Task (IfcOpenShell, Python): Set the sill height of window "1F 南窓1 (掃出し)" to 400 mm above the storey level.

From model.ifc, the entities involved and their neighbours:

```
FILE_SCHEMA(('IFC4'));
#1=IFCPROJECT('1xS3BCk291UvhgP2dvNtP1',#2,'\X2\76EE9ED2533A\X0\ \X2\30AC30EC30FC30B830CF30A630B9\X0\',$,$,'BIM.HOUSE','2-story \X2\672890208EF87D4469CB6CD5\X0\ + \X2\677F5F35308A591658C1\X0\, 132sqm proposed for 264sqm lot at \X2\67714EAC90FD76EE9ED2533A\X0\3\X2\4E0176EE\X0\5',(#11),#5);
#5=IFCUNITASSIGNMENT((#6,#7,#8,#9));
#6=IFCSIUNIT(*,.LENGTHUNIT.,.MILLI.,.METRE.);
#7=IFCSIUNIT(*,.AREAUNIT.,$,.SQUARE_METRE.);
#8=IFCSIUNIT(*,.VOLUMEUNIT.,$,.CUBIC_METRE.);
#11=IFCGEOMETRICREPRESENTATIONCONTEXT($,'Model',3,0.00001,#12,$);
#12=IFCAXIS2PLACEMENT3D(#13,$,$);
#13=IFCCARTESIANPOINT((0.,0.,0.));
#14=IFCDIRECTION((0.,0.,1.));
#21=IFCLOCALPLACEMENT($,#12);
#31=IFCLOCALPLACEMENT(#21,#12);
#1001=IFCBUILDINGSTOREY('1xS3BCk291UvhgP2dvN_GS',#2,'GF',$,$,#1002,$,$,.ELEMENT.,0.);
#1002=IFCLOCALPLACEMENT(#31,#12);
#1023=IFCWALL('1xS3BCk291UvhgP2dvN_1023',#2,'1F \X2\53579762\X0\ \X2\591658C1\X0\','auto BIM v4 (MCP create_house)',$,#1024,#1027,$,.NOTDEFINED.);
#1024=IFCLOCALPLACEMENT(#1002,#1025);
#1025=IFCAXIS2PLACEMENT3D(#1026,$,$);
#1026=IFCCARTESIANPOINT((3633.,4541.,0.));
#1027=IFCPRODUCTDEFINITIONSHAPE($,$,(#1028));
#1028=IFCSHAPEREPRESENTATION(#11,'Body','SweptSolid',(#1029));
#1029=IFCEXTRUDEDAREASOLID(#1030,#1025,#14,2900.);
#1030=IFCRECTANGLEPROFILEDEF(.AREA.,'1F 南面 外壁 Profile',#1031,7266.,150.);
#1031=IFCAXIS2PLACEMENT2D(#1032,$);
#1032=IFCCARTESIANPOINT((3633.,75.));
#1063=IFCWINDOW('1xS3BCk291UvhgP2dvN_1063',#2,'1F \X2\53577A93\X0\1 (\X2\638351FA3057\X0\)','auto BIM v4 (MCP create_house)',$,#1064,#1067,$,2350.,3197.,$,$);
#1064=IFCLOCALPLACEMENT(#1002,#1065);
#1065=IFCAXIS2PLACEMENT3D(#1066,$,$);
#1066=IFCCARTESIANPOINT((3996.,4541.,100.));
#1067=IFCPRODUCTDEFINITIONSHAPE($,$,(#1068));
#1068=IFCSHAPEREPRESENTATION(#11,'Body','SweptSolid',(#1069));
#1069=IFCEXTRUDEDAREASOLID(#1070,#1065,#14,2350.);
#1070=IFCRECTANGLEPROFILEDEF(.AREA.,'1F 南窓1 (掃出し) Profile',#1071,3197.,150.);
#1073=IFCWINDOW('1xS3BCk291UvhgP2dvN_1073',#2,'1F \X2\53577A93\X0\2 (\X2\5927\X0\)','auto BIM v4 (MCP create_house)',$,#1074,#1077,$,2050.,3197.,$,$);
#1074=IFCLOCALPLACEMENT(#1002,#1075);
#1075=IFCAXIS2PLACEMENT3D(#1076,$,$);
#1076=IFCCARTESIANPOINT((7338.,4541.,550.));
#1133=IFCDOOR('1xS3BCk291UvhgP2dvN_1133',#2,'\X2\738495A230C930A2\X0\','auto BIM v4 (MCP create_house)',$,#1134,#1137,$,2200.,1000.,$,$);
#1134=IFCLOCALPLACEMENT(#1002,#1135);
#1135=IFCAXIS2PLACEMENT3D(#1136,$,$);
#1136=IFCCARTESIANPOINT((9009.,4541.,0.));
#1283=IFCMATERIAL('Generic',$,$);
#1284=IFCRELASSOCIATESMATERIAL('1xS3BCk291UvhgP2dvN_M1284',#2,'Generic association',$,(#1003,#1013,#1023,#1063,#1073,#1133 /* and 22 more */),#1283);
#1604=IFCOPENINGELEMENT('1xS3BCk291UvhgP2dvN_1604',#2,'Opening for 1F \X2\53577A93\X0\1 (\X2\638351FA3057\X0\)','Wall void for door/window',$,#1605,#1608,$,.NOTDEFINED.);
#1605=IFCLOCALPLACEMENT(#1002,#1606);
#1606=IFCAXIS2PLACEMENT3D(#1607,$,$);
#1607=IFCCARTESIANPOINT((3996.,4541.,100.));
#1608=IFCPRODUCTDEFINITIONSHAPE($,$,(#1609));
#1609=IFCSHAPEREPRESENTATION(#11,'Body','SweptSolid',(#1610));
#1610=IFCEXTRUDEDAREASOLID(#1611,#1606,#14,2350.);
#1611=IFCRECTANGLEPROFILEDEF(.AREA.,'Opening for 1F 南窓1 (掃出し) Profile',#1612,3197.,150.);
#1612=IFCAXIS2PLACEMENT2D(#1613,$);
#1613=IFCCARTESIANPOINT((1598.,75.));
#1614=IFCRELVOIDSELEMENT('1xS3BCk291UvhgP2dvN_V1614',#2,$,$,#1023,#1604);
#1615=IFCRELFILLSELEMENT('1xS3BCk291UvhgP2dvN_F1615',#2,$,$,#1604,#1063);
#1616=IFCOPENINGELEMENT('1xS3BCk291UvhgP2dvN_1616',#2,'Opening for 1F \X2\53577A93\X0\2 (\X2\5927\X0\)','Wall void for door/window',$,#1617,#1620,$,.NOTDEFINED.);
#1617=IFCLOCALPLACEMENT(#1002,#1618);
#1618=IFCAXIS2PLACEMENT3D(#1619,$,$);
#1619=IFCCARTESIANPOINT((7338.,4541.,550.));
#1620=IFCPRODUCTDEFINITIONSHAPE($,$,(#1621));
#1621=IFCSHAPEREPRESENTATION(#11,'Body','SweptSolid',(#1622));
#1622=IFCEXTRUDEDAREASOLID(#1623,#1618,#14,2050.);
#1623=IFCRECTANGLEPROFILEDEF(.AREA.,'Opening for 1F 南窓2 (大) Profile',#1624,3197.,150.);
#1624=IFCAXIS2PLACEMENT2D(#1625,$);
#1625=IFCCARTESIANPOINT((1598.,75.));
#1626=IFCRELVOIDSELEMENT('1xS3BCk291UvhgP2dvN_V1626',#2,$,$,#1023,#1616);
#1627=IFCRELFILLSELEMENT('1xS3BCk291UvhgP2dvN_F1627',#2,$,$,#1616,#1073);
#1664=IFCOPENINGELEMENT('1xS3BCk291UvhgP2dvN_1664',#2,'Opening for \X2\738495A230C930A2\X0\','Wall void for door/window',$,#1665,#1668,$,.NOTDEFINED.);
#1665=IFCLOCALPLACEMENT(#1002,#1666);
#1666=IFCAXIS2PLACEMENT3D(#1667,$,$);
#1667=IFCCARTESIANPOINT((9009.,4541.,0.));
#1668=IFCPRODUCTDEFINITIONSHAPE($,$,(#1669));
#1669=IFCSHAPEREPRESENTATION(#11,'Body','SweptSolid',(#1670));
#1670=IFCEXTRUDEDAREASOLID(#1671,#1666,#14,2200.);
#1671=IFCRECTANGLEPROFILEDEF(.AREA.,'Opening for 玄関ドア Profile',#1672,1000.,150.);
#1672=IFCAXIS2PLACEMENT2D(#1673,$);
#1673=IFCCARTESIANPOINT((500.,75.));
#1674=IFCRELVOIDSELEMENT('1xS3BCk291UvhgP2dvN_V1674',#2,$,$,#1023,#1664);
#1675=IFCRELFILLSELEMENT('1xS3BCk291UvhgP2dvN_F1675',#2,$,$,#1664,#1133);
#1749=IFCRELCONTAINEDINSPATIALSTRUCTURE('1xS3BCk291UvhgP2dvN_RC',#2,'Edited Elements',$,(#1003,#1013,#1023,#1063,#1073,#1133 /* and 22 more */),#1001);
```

```python
import numpy as np
import ifcopenshell
import ifcopenshell.api.geometry
import ifcopenshell.geom
import ifcopenshell.util.element
import ifcopenshell.util.placement
import ifcopenshell.util.shape
import ifcopenshell.util.unit

model = ifcopenshell.open("model.ifc")
unit_scale = ifcopenshell.util.unit.calculate_unit_scale(model)

window = model.by_id(1063)
opening = window.FillsVoids[0].RelatingOpeningElement
storey = ifcopenshell.util.element.get_container(window, ifc_class="IfcBuildingStorey")
level = ifcopenshell.util.placement.get_local_placement(storey.ObjectPlacement)[2, 3]

# The opening's origin need not be at the sill, so measure its lowest point.
shape = ifcopenshell.geom.create_shape(ifcopenshell.geom.settings(), opening)
bottom = ifcopenshell.util.shape.get_shape_bottom_elevation(shape, shape.geometry) / unit_scale
dz = level + 400.0 - bottom

shift = np.array([0.0, 0.0, dz])
# The window is not placed relative to its opening, so move both.
for product in (opening, window):
    matrix = ifcopenshell.util.placement.get_local_placement(product.ObjectPlacement)
    matrix[:3, 3] += shift
    ifcopenshell.api.geometry.edit_object_placement(model, product=product, matrix=matrix, is_si=False)

print(f"moved by {dz * unit_scale:+.3f} m")

model.write("model_rev.ifc")
```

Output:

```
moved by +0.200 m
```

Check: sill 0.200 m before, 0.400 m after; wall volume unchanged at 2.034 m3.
